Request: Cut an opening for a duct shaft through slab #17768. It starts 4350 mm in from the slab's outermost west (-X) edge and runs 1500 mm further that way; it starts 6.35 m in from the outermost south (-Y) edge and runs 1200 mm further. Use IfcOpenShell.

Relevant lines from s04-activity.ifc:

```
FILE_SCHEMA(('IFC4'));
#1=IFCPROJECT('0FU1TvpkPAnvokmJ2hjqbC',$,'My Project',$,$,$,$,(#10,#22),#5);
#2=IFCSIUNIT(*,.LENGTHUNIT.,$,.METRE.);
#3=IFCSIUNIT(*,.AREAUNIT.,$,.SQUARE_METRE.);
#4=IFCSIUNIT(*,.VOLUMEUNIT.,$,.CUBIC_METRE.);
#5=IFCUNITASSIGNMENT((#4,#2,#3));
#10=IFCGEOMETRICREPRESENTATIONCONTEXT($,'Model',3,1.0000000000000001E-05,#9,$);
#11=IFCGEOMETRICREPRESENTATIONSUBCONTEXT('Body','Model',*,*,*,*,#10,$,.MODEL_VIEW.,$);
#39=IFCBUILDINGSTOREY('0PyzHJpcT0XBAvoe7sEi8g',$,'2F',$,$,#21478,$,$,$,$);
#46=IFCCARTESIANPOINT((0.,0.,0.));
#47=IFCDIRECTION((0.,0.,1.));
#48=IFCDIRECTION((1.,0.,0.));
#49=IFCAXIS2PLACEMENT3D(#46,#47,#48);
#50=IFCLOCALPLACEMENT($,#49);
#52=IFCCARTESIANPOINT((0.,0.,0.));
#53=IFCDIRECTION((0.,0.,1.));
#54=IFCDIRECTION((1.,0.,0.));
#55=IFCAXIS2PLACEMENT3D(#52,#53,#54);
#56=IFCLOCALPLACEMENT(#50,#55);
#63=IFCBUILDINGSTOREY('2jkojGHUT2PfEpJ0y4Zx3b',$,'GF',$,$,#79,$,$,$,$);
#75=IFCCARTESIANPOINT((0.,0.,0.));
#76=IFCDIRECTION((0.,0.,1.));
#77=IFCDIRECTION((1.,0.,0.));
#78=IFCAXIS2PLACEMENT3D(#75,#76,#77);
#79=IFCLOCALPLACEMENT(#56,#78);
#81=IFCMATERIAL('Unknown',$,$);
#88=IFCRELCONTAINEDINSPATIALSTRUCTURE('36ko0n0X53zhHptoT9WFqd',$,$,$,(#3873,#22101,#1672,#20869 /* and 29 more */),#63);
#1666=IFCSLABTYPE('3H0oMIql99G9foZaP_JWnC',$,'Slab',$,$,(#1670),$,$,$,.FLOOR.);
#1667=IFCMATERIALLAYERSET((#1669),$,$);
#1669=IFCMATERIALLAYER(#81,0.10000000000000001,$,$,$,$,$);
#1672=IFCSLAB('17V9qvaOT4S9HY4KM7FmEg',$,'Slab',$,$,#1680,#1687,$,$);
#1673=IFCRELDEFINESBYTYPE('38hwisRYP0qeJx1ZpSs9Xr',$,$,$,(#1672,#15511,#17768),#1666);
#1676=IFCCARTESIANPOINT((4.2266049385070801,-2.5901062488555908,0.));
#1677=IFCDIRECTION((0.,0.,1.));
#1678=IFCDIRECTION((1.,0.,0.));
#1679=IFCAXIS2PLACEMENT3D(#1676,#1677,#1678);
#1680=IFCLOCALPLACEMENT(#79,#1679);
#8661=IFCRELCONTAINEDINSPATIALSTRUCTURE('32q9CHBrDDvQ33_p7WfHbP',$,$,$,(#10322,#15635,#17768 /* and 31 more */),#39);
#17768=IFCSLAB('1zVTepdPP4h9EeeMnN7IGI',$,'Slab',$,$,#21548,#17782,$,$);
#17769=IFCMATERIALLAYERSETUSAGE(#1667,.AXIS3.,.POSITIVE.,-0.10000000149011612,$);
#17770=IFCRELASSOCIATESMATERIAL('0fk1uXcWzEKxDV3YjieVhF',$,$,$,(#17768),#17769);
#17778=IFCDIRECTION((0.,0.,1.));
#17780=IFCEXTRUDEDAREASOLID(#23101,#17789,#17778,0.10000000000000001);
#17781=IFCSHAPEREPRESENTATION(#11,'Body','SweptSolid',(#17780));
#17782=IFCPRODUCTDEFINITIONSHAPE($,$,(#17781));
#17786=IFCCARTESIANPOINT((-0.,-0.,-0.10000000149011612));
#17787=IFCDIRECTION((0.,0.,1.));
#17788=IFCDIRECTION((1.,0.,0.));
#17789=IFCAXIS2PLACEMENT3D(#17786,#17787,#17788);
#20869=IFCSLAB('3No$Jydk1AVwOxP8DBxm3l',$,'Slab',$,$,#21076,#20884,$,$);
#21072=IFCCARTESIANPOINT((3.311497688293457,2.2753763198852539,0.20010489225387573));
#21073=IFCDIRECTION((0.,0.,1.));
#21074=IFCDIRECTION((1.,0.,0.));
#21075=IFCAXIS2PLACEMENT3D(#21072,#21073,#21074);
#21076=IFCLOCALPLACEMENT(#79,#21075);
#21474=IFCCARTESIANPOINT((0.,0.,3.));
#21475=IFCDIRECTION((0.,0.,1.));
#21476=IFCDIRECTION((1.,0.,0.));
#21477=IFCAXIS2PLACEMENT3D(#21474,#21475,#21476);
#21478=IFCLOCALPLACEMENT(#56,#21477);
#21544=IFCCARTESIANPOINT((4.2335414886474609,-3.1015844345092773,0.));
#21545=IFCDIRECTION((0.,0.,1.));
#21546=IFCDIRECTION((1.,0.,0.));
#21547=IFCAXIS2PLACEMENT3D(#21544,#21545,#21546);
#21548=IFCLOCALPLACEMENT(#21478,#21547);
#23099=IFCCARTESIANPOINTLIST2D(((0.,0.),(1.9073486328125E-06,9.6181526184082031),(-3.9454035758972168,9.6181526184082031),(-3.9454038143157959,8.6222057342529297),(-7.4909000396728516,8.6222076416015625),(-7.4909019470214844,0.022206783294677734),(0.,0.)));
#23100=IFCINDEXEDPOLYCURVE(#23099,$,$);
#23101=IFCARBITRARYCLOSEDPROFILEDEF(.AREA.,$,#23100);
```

```python
import numpy as np
import ifcopenshell
import ifcopenshell.api.feature
import ifcopenshell.api.geometry
import ifcopenshell.api.root
import ifcopenshell.geom
import ifcopenshell.util.placement
import ifcopenshell.util.representation
import ifcopenshell.util.shape
import ifcopenshell.util.unit

model = ifcopenshell.open("s04-activity.ifc")
unit_scale = ifcopenshell.util.unit.calculate_unit_scale(model)
settings = ifcopenshell.geom.settings()


def volume(element):
    """Net volume in cubic metres, openings subtracted."""
    shape = ifcopenshell.geom.create_shape(settings, element)
    return ifcopenshell.util.shape.get_volume(shape.geometry)


slab = model.by_guid("1zVTepdPP4h9EeeMnN7IGI")
before = volume(slab)

# Extent in the slab's own axes, in metres. The edges named are its -X and -Y sides.
slab_shape = ifcopenshell.geom.create_shape(settings, slab)
vertices = ifcopenshell.util.shape.get_vertices(slab_shape.geometry)
x_min, y_min, bottom = vertices.min(axis=0)
top = vertices[:, 2].max()

opening = ifcopenshell.api.root.create_entity(model, ifc_class="IfcOpeningElement", name="Duct shaft opening", predefined_type="OPENING")
context = ifcopenshell.util.representation.get_context(model, "Model", "Body", "MODEL_VIEW")
width, depth = 1.5, 1.2
outline = [(0.0, 0.0), (width, 0.0), (width, depth), (0.0, depth), (0.0, 0.0)]
# Overshoot both faces by 50 mm so the cut is clean.
shape = ifcopenshell.api.geometry.add_slab_representation(
    model, context=context, depth=top - bottom + 0.1, polyline=outline
)
ifcopenshell.api.geometry.assign_representation(model, product=opening, representation=shape)

matrix = ifcopenshell.util.placement.get_local_placement(slab.ObjectPlacement)
matrix[:, 3] = matrix @ np.append(np.array([x_min + 4.35, y_min + 6.35, bottom - 0.05]) / unit_scale, 1.0)
ifcopenshell.api.geometry.edit_object_placement(model, product=opening, matrix=matrix, is_si=False)
ifcopenshell.api.feature.add_feature(model, feature=opening, element=slab)

after = volume(slab)

print(f"slab volume {before:.3f} -> {after:.3f} m3")

model.write("s04-activity_v2.ifc")
```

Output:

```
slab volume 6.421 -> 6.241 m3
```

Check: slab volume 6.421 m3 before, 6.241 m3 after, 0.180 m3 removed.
